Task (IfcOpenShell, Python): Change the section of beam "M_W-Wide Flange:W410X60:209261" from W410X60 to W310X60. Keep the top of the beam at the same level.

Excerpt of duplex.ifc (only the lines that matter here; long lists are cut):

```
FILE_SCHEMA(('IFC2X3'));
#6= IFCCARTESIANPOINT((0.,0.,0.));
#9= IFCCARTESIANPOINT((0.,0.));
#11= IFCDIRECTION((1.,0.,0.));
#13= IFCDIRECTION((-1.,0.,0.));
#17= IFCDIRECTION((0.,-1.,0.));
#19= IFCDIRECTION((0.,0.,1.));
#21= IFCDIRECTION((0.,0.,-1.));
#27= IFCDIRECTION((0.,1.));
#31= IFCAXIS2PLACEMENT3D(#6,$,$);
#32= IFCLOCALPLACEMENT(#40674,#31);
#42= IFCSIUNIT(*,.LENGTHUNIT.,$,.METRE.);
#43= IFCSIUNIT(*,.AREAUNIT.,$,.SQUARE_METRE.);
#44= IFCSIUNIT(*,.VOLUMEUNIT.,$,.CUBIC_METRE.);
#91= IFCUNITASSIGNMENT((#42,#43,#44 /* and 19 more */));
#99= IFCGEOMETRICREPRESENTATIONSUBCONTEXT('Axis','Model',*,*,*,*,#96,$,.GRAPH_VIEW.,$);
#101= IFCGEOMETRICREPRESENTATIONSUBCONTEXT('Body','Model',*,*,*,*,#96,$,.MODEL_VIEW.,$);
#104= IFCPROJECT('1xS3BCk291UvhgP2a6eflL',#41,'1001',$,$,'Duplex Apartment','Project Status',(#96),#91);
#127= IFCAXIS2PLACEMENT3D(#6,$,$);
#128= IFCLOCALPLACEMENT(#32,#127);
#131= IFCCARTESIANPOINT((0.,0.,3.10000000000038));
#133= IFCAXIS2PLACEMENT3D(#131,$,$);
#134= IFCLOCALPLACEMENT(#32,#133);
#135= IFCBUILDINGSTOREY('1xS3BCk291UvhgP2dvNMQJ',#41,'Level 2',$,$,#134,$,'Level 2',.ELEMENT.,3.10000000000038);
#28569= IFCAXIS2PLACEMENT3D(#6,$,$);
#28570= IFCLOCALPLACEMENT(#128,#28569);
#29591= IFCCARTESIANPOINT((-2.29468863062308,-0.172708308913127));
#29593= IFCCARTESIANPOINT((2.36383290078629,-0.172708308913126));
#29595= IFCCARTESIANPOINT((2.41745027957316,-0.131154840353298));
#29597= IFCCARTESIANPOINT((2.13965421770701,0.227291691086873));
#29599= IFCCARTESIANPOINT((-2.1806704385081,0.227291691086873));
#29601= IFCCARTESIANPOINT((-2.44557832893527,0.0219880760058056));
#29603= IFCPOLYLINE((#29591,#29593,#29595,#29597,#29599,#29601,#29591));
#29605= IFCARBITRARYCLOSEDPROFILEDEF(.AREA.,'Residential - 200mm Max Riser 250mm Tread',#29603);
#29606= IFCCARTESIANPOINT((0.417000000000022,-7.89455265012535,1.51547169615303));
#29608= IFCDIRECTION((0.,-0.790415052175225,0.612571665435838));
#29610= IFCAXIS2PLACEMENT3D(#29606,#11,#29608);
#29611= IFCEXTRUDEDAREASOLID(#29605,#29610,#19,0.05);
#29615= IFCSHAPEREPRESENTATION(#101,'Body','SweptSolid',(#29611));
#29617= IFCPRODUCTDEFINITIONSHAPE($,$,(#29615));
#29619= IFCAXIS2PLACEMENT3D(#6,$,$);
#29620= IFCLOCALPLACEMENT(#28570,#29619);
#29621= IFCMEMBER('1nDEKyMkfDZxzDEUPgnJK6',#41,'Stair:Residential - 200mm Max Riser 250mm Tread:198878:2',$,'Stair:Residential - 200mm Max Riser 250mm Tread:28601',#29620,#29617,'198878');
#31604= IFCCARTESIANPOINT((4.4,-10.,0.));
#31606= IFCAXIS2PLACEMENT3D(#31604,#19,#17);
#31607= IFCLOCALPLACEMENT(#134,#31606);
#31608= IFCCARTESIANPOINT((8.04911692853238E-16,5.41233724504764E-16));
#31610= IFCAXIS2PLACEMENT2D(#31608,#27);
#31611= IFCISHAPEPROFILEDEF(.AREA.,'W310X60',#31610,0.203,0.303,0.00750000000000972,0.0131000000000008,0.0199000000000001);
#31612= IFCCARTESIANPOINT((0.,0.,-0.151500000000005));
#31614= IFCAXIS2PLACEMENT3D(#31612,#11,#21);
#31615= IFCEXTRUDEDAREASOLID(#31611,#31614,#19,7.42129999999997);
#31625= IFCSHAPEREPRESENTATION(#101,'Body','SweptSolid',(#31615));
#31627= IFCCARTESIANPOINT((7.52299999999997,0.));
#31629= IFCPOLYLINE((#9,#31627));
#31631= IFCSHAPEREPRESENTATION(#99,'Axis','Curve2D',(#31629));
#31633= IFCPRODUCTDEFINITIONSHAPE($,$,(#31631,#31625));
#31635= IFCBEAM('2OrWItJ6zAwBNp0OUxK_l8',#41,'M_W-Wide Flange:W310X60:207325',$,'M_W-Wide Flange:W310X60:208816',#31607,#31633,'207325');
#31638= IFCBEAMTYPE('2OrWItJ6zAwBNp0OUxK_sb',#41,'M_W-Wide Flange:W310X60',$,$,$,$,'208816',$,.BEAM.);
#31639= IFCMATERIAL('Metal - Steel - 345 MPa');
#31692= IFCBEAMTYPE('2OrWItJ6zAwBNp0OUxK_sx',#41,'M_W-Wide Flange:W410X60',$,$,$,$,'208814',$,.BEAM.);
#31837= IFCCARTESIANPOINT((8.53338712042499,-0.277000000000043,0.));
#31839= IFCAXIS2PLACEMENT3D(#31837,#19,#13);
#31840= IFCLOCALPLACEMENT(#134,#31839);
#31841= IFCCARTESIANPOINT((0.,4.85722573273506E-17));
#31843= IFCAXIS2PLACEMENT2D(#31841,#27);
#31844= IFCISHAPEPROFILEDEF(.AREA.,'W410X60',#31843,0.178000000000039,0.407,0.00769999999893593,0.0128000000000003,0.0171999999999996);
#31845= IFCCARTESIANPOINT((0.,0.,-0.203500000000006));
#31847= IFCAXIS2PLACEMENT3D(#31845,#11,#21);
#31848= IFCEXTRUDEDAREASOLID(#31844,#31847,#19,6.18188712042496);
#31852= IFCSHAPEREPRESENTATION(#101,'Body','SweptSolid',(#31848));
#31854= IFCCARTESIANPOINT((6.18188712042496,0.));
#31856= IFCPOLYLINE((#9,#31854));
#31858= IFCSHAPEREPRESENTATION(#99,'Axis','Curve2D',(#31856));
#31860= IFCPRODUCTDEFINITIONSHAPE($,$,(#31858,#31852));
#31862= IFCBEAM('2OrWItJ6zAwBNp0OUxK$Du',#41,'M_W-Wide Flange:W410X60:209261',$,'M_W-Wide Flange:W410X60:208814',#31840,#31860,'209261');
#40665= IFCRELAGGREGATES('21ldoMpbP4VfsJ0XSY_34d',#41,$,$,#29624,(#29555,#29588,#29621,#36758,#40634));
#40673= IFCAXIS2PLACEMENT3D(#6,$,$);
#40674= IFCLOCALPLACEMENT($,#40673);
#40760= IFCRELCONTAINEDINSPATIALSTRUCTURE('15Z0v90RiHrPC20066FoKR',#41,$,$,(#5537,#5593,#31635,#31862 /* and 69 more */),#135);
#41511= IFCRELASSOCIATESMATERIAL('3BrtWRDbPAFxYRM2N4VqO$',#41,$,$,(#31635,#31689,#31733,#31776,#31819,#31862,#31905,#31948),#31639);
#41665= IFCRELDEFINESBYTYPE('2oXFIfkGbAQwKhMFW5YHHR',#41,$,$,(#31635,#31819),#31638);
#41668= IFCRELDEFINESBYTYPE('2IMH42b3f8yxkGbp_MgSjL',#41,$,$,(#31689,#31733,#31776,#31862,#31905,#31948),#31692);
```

```python
import ifcopenshell
import ifcopenshell.api.type
import ifcopenshell.util.element
import ifcopenshell.util.representation

model = ifcopenshell.open("duplex.ifc")

member = model.by_guid("2OrWItJ6zAwBNp0OUxK$Du")
source = next(p for p in model.by_type("IfcIShapeProfileDef") if p.ProfileName == "W310X60")

body = ifcopenshell.util.representation.get_representation(member, "Model", "Body")
solid = body.Items[0]
old_profile = solid.SweptArea

# Copy the section's sizes but keep this member's own profile position.
profile = ifcopenshell.util.element.copy(model, source)
# Profiles are centred, so shift by half the change in depth to hold the top.
shift = (old_profile.OverallDepth - profile.OverallDepth) / 2
x, y = old_profile.Position.Location.Coordinates
up = (-1.0, 0.0)  # upwards, in the solid's own plane
location = model.createIfcCartesianPoint((x + up[0] * shift, y + up[1] * shift))
profile.Position = model.createIfcAxis2Placement2D(location, old_profile.Position.RefDirection)
solid.SweptArea = profile
if not model.get_total_inverses(old_profile):
    ifcopenshell.util.element.remove_deep2(model, old_profile)

new_type = model.by_guid("2OrWItJ6zAwBNp0OUxK_sb")
ifcopenshell.api.type.assign_type(
    model, related_objects=[member], relating_type=new_type, should_map_representations=False
)
member.Name = member.Name.replace("W410X60", "W310X60")
member.ObjectType = "M_W-Wide Flange:W310X60:208814"

print(solid.SweptArea)

model.write("duplex_v2.ifc")
```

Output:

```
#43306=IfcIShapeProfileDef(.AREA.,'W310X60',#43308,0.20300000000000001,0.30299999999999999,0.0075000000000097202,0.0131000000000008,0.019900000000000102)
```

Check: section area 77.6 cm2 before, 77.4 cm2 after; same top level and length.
